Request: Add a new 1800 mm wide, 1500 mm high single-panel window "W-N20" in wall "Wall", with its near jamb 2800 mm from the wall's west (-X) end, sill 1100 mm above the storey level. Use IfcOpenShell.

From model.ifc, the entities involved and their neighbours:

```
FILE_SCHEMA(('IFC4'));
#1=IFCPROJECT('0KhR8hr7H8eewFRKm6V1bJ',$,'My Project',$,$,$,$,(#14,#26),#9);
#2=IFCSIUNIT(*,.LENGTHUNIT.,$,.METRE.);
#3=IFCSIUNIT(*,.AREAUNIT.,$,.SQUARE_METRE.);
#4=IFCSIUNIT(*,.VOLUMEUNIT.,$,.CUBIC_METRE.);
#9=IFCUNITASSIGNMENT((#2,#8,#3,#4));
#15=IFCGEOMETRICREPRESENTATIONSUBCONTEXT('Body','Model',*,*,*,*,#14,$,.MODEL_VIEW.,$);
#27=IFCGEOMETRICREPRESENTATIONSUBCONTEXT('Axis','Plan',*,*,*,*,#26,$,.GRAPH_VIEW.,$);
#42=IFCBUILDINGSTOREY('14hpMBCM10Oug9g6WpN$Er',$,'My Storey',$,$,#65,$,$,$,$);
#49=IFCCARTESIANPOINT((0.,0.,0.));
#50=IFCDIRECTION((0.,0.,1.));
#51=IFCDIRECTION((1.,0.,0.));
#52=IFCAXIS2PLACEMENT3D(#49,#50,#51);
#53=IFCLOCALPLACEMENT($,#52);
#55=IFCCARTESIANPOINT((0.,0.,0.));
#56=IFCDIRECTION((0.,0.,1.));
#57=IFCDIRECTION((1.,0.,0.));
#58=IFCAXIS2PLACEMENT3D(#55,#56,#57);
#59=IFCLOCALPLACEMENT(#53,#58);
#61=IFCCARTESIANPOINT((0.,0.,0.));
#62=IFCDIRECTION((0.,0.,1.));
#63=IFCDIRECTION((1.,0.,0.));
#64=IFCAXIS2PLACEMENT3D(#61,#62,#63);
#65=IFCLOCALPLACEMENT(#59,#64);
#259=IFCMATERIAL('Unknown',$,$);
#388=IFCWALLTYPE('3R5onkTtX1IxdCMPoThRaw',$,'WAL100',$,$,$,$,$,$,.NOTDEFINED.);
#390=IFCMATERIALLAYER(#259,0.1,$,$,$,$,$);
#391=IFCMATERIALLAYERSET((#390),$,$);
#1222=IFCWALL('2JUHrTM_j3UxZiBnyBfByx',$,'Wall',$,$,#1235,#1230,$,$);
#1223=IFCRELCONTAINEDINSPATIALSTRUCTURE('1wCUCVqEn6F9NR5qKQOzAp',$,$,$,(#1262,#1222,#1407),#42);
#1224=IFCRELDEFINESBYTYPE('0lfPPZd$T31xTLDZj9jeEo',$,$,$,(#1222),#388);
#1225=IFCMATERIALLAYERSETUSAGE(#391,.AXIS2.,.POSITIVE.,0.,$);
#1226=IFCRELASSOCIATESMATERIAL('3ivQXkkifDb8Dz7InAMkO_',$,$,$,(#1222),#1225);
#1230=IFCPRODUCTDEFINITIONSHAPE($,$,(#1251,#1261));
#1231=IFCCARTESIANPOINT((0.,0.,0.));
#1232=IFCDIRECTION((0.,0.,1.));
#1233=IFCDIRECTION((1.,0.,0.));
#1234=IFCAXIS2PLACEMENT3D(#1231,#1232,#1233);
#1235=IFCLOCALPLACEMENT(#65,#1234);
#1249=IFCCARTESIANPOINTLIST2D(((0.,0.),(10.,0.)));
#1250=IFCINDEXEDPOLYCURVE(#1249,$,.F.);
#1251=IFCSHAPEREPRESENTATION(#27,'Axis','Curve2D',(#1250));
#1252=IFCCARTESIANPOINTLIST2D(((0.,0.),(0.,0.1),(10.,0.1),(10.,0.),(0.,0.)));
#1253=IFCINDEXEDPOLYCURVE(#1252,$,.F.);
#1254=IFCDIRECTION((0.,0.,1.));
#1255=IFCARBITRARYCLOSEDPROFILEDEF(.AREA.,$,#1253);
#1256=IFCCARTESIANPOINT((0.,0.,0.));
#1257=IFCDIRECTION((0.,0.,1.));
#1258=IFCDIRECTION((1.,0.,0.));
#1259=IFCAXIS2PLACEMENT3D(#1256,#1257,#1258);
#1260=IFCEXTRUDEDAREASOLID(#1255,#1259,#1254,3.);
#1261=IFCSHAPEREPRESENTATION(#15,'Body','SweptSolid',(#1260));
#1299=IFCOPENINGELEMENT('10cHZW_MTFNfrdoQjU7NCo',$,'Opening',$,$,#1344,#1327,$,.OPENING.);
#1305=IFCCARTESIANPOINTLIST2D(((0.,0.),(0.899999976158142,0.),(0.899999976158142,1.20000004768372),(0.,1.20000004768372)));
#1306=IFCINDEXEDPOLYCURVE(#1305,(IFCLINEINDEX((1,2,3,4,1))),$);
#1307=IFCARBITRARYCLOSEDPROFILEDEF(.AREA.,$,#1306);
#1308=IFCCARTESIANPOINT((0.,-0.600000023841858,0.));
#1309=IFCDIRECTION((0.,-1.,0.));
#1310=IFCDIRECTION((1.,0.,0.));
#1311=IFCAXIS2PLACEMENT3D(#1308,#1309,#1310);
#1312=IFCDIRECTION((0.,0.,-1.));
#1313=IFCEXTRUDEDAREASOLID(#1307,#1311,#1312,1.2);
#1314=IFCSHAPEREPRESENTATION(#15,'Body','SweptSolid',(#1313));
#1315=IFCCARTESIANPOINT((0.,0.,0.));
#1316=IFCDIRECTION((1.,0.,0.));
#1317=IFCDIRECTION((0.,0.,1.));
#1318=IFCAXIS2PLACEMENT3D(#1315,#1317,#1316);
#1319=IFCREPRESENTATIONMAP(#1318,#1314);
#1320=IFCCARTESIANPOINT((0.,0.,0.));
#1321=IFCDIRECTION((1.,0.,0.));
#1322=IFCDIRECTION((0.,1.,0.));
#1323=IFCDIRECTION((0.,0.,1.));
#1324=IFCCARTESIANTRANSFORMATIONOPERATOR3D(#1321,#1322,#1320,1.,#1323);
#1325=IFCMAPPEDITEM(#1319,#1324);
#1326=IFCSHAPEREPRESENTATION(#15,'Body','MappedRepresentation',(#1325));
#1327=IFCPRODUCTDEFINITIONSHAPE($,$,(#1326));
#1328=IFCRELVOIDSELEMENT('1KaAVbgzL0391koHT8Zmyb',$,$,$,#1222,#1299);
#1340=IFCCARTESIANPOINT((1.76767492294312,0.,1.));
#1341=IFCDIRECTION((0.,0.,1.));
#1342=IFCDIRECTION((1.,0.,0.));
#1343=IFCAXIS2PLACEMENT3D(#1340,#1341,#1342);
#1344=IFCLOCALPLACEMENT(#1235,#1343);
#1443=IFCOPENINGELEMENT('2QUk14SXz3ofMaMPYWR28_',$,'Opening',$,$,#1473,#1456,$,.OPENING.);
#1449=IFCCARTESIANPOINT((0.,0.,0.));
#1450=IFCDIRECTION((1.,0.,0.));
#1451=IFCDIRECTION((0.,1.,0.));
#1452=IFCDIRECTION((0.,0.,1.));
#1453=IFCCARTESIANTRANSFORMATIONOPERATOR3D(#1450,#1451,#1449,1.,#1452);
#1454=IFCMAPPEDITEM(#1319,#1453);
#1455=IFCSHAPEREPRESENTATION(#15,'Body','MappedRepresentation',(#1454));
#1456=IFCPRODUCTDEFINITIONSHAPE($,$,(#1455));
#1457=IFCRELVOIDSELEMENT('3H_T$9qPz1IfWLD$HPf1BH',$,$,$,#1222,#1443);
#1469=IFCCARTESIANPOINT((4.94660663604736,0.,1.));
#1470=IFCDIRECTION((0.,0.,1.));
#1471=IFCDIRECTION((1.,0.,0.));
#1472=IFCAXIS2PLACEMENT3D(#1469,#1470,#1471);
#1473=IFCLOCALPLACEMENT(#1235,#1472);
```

```python
import numpy as np
import ifcopenshell
import ifcopenshell.api.feature
import ifcopenshell.api.geometry
import ifcopenshell.api.root
import ifcopenshell.api.spatial
import ifcopenshell.geom
import ifcopenshell.util.element
import ifcopenshell.util.placement
import ifcopenshell.util.representation
import ifcopenshell.util.shape
import ifcopenshell.util.unit

model = ifcopenshell.open("model.ifc")
unit_scale = ifcopenshell.util.unit.calculate_unit_scale(model)
settings = ifcopenshell.geom.settings()


def volume(element):
    """Net volume in cubic metres, openings subtracted."""
    shape = ifcopenshell.geom.create_shape(settings, element)
    return ifcopenshell.util.shape.get_volume(shape.geometry)


wall = model.by_guid("2JUHrTM_j3UxZiBnyBfByx")
storey = ifcopenshell.util.element.get_container(wall, ifc_class="IfcBuildingStorey")
context = ifcopenshell.util.representation.get_context(model, "Model", "Body", "MODEL_VIEW")
before = volume(wall)

width, height, from_end, sill = 1.8, 1.5, 2.8, 1.1  # metres

# The wall runs along its own X axis, and the end named is its -X end.
wall_shape = ifcopenshell.geom.create_shape(settings, wall)
x, y, z = ifcopenshell.util.shape.get_vertices(wall_shape.geometry).T
start = x.min() + from_end
face, thickness = float(y.min()), float(y.max() - y.min())
wall_matrix = ifcopenshell.util.placement.get_local_placement(wall.ObjectPlacement)
level = ifcopenshell.util.placement.get_local_placement(storey.ObjectPlacement)[2, 3]


def in_wall(x, y):
    """Placement at x, y metres in the wall's axes, at sill height."""
    matrix = wall_matrix.copy()
    matrix[:, 3] = wall_matrix @ np.array([x / unit_scale, y / unit_scale, 0.0, 1.0])
    matrix[2, 3] = level + sill / unit_scale
    return matrix


# Opening: a box that overshoots both wall faces by 50 mm.
opening = ifcopenshell.api.root.create_entity(model, ifc_class="IfcOpeningElement", predefined_type="OPENING")
box = ifcopenshell.api.geometry.add_wall_representation(
    model, context=context, length=width, height=height, thickness=thickness + 0.1
)
ifcopenshell.api.geometry.assign_representation(model, product=opening, representation=box)
ifcopenshell.api.geometry.edit_object_placement(model, product=opening, matrix=in_wall(start, face - 0.05), is_si=False)
ifcopenshell.api.feature.add_feature(model, feature=opening, element=wall)

window = ifcopenshell.api.root.create_entity(model, ifc_class="IfcWindow", name="W-N20", predefined_type="WINDOW")
window.OverallWidth, window.OverallHeight = width / unit_scale, height / unit_scale
window.PartitioningType = "SINGLE_PANEL"
body = ifcopenshell.api.geometry.add_window_representation(
    model,
    context=context,
    overall_width=window.OverallWidth,
    overall_height=window.OverallHeight,
    partition_type="SINGLE_PANEL",
)
ifcopenshell.api.geometry.assign_representation(model, product=window, representation=body)
ifcopenshell.api.spatial.assign_container(model, products=[window], relating_structure=storey)
ifcopenshell.api.feature.add_filling(model, opening=opening, element=window)

# Centre the window in the wall's thickness.
ifcopenshell.api.geometry.edit_object_placement(model, product=window, matrix=in_wall(start, face), is_si=False)
window_shape = ifcopenshell.geom.create_shape(settings, window)
depth = ifcopenshell.util.shape.get_vertices(window_shape.geometry)[:, 1]
offset = face + thickness / 2 - (depth.min() + depth.max()) / 2
ifcopenshell.api.geometry.edit_object_placement(model, product=window, matrix=in_wall(start, offset), is_si=False)

after = volume(wall)

print(f"wall volume {before:.3f} -> {after:.3f} m3")

model.write("model-out.ifc")
```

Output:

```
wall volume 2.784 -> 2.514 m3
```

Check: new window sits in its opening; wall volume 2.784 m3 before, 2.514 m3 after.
